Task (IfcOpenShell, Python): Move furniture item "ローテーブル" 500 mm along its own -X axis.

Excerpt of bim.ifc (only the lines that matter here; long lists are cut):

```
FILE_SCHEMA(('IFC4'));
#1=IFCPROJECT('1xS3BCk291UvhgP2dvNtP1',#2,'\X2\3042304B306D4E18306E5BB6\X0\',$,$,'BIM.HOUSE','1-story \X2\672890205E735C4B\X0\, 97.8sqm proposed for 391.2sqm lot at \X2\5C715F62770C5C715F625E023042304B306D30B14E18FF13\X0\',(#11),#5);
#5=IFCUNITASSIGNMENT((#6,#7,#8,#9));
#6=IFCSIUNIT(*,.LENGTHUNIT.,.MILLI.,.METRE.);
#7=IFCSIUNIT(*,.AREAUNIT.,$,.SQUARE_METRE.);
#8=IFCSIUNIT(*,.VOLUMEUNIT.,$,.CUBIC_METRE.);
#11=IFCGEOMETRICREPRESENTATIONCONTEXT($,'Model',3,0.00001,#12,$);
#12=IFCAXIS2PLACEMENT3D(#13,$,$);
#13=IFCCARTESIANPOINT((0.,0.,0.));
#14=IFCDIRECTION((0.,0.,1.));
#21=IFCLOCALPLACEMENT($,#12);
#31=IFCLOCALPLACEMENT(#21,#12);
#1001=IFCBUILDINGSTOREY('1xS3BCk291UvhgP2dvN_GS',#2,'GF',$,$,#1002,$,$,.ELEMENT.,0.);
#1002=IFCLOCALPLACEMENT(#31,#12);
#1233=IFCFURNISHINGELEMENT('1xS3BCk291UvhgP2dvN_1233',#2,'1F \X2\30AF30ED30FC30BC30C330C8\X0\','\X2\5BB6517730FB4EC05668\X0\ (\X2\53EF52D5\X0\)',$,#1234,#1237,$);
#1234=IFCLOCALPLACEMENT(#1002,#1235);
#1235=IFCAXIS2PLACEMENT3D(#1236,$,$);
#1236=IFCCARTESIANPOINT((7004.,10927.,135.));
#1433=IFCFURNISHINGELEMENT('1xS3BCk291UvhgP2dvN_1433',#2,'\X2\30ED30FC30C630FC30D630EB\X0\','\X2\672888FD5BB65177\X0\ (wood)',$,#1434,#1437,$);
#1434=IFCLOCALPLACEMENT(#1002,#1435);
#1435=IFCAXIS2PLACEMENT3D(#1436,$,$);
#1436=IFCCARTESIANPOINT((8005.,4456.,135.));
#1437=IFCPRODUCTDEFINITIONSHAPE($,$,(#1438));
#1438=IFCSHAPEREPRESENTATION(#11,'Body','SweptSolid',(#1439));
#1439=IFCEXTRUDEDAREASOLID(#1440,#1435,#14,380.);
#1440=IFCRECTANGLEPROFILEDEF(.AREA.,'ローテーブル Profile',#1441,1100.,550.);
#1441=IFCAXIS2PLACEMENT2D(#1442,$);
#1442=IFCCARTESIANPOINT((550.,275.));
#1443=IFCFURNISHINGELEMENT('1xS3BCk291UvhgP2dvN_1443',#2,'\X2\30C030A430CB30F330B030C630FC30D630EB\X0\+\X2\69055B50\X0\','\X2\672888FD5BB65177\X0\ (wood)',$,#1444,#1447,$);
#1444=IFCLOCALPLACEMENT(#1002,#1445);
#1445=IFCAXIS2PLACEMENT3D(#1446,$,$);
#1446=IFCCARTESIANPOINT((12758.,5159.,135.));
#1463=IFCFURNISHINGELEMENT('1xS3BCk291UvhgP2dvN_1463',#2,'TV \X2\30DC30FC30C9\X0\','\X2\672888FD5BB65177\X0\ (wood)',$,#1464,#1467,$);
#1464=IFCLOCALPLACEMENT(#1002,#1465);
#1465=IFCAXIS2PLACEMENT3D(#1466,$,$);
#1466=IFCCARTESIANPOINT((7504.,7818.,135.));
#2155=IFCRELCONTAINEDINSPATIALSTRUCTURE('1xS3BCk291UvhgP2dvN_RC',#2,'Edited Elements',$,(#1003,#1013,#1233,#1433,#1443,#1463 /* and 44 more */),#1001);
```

```python
import ifcopenshell
import ifcopenshell.api.geometry
import ifcopenshell.util.placement
import ifcopenshell.util.unit

model = ifcopenshell.open("bim.ifc")
unit_scale = ifcopenshell.util.unit.calculate_unit_scale(model)

item = model.by_guid("1xS3BCk291UvhgP2dvN_1433")
matrix = ifcopenshell.util.placement.get_local_placement(item.ObjectPlacement)
matrix[:3, 3] -= matrix[:3, 0] * 0.5 / unit_scale
ifcopenshell.api.geometry.edit_object_placement(model, product=item, matrix=matrix, is_si=False)

print(ifcopenshell.util.placement.get_local_placement(item.ObjectPlacement).round(3) + 0.0)

model.write("bim-out.ifc")
```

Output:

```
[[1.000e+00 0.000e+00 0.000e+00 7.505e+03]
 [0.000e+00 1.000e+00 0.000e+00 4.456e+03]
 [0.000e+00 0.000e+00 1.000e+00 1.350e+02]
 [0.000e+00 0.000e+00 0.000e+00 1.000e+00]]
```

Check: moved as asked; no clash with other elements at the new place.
